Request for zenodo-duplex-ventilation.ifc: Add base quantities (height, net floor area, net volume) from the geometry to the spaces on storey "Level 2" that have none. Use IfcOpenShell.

First a look at what the model holds.

```python
import ifcopenshell
import ifcopenshell.util.element
import ifcopenshell.util.unit

model = ifcopenshell.open("zenodo-duplex-ventilation.ifc")
print(model.schema)
for unit_type in ("LENGTHUNIT", "AREAUNIT", "VOLUMEUNIT"):
    print(unit_type, ifcopenshell.util.unit.calculate_unit_scale(model, unit_type))
storey = next(s for s in model.by_type("IfcBuildingStorey") if s.Name == "Level 2")
spaces = [e for e in ifcopenshell.util.element.get_decomposition(storey) if e.is_a("IfcSpace")]
for e in sorted(spaces, key=lambda e: e.id()):
    print(e.id(), e.is_a(), e.Name, list(ifcopenshell.util.element.get_psets(e, qtos_only=True)), sep=" | ")
```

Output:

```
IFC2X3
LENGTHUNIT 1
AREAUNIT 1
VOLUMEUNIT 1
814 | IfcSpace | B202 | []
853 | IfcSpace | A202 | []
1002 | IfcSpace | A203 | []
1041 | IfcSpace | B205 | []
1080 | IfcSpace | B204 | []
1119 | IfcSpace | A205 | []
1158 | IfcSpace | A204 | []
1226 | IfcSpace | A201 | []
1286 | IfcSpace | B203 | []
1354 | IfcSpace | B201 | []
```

```python
import ifcopenshell
import ifcopenshell.api.pset
import ifcopenshell.geom
import ifcopenshell.util.element
import ifcopenshell.util.shape
import ifcopenshell.util.unit

model = ifcopenshell.open("zenodo-duplex-ventilation.ifc")
unit_scale = ifcopenshell.util.unit.calculate_unit_scale(model)
area_scale = ifcopenshell.util.unit.calculate_unit_scale(model, "AREAUNIT")
volume_scale = ifcopenshell.util.unit.calculate_unit_scale(model, "VOLUMEUNIT")
settings = ifcopenshell.geom.settings()

storey = next(s for s in model.by_type("IfcBuildingStorey") if s.Name == "Level 2")
spaces = [e for e in ifcopenshell.util.element.get_decomposition(storey) if e.is_a("IfcSpace")]

for e in sorted(spaces, key=lambda e: e.id()):
    if ifcopenshell.util.element.get_psets(e, qtos_only=True, should_inherit=False):
        continue
    # Geometry comes back in metres, in the element's own axes.
    shape = ifcopenshell.geom.create_shape(settings, e)
    values = {
        "Height": ifcopenshell.util.shape.get_z(shape.geometry) / unit_scale,
        "NetFloorArea": ifcopenshell.util.shape.get_footprint_area(shape.geometry) / area_scale,
        "NetVolume": ifcopenshell.util.shape.get_volume(shape.geometry) / volume_scale,
    }
    qto = ifcopenshell.api.pset.add_qto(model, product=e, name="BaseQuantities")
    ifcopenshell.api.pset.edit_qto(model, qto=qto, properties=values)
    print(e.id(), {k: round(v, 3) for k, v in values.items()})

model.write("zenodo-duplex-ventilation-out.ifc")
```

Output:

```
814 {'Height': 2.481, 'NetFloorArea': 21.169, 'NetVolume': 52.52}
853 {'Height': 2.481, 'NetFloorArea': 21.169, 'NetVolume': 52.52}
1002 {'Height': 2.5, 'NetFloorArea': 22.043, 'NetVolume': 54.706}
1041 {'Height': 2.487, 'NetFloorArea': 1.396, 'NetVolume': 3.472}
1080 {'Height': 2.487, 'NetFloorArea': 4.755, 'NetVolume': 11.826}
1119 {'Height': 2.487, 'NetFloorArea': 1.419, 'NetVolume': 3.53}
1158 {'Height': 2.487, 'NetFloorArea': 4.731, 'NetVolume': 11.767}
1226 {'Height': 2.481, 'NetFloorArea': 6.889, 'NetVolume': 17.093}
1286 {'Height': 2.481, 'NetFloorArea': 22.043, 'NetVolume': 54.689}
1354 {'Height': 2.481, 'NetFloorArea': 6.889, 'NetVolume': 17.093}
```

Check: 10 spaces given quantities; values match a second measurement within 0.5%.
